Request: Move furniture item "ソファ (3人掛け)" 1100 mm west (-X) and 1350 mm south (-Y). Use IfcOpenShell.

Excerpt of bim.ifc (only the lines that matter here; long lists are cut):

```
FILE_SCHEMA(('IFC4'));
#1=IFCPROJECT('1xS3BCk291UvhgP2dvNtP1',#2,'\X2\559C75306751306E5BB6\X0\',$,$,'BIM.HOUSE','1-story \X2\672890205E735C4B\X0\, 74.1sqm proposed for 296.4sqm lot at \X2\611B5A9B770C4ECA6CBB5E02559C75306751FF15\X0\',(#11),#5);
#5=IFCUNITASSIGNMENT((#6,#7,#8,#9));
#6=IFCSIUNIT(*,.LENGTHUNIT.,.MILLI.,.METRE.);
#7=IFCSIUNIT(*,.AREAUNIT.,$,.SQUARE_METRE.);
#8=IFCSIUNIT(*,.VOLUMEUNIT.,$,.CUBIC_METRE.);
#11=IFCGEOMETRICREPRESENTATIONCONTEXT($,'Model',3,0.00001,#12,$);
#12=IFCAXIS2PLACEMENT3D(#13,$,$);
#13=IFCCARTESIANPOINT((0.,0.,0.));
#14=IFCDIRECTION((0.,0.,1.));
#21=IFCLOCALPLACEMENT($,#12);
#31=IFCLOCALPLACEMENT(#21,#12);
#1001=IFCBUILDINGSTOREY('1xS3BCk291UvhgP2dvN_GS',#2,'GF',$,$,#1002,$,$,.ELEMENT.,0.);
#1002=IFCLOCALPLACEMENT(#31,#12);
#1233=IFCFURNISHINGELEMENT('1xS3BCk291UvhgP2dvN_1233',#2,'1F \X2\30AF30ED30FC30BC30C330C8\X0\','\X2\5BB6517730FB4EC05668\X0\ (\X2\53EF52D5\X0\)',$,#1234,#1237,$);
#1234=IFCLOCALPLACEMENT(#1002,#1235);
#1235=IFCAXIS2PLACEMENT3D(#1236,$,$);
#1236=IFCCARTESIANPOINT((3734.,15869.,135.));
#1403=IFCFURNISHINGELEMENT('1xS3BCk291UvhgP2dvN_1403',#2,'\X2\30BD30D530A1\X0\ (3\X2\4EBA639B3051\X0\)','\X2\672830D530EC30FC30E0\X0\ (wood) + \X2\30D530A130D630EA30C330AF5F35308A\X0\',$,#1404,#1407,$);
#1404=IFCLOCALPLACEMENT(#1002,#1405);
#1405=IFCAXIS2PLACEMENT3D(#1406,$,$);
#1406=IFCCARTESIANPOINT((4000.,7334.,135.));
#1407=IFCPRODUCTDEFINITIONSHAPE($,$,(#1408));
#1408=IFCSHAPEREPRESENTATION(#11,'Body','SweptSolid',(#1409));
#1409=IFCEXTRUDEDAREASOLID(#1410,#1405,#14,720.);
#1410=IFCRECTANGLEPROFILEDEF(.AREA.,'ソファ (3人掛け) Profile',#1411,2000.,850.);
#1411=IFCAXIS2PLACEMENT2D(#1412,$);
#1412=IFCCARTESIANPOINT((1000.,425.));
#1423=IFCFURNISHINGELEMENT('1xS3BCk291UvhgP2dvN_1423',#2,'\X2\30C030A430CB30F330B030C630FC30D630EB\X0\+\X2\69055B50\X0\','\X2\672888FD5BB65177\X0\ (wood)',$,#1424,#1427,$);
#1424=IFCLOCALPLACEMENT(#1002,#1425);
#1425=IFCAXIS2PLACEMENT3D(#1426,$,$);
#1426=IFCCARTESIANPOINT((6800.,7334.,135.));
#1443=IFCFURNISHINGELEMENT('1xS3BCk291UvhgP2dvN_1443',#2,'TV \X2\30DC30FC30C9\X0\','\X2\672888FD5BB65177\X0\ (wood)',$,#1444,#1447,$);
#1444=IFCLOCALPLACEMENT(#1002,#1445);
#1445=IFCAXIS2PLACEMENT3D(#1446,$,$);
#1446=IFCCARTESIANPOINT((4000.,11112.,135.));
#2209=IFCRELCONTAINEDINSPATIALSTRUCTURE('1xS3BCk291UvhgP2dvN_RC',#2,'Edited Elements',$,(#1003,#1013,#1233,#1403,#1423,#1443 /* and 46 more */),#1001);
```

```python
import ifcopenshell
import ifcopenshell.api.geometry
import ifcopenshell.util.placement
import ifcopenshell.util.unit

model = ifcopenshell.open("bim.ifc")
unit_scale = ifcopenshell.util.unit.calculate_unit_scale(model)

item = model.by_guid("1xS3BCk291UvhgP2dvN_1403")
matrix = ifcopenshell.util.placement.get_local_placement(item.ObjectPlacement)
matrix[0, 3] -= 1.1 / unit_scale
matrix[1, 3] -= 1.35 / unit_scale
ifcopenshell.api.geometry.edit_object_placement(model, product=item, matrix=matrix, is_si=False)

print(ifcopenshell.util.placement.get_local_placement(item.ObjectPlacement).round(3) + 0.0)

model.write("bim_edited.ifc")
```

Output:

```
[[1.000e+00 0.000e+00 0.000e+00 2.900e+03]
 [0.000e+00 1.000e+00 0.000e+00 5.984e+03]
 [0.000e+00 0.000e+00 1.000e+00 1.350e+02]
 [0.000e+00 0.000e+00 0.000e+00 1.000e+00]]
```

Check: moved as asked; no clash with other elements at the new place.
